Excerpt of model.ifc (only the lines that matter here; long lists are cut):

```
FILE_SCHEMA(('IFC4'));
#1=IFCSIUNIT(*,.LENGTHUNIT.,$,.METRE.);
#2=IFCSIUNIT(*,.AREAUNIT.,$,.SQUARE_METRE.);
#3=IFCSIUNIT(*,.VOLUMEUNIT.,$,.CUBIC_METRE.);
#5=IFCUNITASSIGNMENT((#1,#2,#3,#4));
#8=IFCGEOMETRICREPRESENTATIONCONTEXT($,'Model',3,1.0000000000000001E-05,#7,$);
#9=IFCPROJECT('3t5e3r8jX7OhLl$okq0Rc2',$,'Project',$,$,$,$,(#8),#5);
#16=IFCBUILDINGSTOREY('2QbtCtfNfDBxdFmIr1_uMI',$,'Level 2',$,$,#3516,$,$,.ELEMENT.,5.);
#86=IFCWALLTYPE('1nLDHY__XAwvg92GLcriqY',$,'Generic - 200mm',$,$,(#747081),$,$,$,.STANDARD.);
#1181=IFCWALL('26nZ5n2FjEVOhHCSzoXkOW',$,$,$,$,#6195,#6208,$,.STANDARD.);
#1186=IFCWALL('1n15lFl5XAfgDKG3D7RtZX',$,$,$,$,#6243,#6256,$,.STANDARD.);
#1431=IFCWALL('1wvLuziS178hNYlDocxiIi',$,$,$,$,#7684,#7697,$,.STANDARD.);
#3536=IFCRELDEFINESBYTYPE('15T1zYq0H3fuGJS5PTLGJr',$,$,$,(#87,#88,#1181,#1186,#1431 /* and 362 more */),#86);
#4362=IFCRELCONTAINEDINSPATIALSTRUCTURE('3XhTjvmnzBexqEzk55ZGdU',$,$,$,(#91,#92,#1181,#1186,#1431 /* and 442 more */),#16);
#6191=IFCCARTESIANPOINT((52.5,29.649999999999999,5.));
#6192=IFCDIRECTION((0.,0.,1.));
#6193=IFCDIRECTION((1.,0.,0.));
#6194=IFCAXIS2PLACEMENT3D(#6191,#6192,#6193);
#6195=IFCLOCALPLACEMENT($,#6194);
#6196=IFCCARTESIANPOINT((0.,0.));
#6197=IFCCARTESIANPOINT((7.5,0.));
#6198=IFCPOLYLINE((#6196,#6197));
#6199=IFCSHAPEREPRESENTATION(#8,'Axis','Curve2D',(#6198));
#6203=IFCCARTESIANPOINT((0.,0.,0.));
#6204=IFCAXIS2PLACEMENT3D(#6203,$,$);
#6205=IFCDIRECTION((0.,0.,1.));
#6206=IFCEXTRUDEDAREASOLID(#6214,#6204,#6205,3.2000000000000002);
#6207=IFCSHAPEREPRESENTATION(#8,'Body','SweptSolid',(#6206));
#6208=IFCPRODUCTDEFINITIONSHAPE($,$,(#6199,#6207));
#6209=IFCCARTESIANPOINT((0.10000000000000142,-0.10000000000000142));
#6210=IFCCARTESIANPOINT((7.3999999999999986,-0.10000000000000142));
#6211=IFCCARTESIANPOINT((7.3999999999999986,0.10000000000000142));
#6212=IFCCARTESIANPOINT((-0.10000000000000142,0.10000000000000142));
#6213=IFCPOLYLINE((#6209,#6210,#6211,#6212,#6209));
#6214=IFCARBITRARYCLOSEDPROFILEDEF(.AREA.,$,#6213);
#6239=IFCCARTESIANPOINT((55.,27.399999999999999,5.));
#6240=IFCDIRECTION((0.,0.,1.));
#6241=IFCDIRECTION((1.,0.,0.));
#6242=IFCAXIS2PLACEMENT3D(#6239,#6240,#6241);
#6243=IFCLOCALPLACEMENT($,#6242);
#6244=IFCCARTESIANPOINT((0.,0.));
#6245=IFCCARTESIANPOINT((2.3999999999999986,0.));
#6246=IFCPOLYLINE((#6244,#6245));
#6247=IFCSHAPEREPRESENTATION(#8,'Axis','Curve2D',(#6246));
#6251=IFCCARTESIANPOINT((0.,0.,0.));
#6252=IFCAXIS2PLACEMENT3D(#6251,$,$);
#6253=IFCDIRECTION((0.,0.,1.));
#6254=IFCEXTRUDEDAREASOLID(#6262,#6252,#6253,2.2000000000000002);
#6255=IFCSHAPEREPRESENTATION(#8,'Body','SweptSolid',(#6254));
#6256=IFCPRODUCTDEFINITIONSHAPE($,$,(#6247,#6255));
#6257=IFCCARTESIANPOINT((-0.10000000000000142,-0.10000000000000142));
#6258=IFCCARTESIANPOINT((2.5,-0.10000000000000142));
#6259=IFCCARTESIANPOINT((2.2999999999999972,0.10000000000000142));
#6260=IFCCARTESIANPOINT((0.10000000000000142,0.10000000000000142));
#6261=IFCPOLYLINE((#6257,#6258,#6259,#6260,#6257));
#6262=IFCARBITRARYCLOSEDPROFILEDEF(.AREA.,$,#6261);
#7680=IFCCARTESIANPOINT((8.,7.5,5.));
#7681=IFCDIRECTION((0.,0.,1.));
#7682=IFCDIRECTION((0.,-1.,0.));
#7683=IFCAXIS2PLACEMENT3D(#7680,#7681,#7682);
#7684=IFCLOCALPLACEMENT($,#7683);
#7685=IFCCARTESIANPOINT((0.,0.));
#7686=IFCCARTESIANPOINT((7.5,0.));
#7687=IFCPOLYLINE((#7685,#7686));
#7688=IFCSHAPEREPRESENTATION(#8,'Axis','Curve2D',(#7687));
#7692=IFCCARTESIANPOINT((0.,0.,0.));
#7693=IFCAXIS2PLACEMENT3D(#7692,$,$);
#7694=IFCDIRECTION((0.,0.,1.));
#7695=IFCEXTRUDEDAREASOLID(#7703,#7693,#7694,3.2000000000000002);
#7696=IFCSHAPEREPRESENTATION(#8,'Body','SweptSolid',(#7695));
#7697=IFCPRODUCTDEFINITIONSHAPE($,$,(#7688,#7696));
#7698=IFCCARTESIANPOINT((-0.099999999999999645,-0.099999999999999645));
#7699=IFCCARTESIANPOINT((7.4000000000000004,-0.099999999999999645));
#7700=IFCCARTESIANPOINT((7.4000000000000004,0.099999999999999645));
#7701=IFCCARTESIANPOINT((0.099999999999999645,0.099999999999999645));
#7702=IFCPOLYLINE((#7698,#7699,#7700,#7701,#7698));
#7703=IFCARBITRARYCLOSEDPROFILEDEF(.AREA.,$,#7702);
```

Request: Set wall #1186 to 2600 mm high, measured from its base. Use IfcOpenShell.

```python
import ifcopenshell
import ifcopenshell.geom
import ifcopenshell.util.shape

model = ifcopenshell.open("model.ifc")
settings = ifcopenshell.geom.settings()


def volume(element):
    """Net volume in cubic metres, openings subtracted."""
    shape = ifcopenshell.geom.create_shape(settings, element)
    return ifcopenshell.util.shape.get_volume(shape.geometry)


wall = model.by_guid("1n15lFl5XAfgDKG3D7RtZX")
before = volume(wall)

body = next(r for r in wall.Representation.Representations if r.RepresentationIdentifier == "Body")
solid = body.Items[0]
old_height = solid.Depth
solid.Depth = 2.6
after = volume(wall)

print(f"height {old_height:g} -> {solid.Depth:g}, volume {before:.3f} -> {after:.3f} m3")

model.write("model-out.ifc")
```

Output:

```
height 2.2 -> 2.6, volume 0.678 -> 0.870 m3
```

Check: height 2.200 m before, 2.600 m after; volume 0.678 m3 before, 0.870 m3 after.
